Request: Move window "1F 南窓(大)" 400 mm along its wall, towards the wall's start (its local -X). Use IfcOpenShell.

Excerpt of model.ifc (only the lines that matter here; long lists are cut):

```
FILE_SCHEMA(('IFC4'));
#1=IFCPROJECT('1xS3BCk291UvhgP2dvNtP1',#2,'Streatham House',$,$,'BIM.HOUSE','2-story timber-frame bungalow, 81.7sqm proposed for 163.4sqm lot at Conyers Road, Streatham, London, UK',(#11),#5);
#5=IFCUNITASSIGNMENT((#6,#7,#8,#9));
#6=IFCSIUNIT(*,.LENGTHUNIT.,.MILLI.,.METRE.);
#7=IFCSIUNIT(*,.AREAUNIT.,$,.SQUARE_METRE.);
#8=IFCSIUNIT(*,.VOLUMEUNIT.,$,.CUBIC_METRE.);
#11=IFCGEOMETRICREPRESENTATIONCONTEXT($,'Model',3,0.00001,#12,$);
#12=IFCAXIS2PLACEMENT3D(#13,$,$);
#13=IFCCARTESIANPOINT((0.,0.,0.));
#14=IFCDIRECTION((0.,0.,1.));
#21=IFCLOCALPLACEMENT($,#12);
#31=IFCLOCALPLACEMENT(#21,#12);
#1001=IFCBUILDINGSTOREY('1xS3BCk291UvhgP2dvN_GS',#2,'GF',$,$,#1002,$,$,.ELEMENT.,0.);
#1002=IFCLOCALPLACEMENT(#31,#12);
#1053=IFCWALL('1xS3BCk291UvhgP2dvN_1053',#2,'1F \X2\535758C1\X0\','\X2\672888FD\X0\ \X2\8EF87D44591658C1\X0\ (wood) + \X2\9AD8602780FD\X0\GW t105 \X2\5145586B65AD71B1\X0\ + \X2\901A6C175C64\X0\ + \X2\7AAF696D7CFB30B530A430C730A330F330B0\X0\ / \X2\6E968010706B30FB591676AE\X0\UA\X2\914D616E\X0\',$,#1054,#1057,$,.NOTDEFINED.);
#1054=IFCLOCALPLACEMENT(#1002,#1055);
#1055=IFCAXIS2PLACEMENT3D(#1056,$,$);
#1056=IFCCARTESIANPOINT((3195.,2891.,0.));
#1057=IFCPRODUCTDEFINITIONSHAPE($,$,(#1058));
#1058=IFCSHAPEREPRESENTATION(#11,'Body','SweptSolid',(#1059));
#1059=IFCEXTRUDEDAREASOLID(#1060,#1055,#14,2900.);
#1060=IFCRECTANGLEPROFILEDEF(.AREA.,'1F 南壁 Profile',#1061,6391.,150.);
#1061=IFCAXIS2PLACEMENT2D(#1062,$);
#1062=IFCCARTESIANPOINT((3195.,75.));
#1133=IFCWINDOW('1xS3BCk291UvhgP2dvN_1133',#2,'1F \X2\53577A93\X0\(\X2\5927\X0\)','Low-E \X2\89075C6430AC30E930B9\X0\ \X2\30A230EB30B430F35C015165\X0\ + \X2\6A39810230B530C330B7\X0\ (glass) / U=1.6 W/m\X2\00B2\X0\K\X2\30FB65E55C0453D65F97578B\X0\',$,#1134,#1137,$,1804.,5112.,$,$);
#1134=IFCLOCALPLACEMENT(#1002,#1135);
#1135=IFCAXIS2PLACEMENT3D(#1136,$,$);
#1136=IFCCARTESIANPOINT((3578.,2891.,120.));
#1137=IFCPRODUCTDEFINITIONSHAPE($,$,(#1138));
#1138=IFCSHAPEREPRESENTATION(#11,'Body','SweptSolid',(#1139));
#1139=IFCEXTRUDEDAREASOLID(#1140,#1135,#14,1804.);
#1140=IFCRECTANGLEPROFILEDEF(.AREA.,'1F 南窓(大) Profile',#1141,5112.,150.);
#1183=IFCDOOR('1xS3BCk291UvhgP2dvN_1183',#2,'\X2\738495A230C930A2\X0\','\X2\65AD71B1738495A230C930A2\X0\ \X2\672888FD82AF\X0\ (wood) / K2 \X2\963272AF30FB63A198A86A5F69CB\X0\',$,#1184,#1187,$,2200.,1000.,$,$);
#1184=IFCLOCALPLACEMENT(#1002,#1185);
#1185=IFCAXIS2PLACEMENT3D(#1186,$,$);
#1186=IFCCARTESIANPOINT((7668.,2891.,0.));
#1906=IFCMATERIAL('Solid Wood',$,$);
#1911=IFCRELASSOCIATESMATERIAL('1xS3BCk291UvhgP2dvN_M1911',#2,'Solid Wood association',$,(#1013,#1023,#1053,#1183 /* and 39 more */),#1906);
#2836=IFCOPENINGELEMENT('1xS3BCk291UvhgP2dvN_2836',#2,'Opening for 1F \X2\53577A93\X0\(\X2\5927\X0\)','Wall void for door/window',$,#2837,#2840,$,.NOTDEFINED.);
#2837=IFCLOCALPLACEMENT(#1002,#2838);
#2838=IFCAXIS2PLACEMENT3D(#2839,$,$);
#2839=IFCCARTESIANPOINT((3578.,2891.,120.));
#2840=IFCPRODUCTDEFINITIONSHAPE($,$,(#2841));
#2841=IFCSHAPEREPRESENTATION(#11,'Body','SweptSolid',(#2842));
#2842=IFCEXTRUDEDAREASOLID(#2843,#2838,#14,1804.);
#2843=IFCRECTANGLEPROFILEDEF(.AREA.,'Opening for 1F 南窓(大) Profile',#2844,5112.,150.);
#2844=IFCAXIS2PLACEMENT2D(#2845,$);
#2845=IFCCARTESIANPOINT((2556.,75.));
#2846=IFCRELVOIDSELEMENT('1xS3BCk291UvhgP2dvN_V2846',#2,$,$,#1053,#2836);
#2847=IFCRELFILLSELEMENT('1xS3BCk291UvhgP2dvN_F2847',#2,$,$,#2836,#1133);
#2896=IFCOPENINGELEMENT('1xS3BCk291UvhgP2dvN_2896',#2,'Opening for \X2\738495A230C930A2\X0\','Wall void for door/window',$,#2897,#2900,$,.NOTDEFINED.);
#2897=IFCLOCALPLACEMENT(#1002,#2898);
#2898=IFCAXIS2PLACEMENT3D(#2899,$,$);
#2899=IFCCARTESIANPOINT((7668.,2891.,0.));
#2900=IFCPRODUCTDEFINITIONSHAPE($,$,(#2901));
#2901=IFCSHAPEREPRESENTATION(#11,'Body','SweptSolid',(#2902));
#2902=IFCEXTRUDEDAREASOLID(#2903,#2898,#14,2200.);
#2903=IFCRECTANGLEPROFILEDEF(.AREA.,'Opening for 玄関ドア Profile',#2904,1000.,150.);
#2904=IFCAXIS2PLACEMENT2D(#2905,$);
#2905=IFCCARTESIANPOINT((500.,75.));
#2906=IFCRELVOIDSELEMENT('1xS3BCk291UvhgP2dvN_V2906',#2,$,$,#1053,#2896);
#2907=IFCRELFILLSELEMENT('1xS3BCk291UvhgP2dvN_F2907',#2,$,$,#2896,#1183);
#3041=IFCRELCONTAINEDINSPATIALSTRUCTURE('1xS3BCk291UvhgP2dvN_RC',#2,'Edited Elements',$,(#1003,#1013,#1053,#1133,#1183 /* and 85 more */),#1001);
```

```python
import ifcopenshell
import ifcopenshell.api.geometry
import ifcopenshell.util.placement
import ifcopenshell.util.unit

model = ifcopenshell.open("model.ifc")
unit_scale = ifcopenshell.util.unit.calculate_unit_scale(model)

window = model.by_id(1133)
opening = window.FillsVoids[0].RelatingOpeningElement
wall = opening.VoidsElements[0].RelatingBuildingElement

wall_matrix = ifcopenshell.util.placement.get_local_placement(wall.ObjectPlacement)
shift = wall_matrix[:3, 0] * -0.4 / unit_scale
before = ifcopenshell.util.placement.get_local_placement(window.ObjectPlacement)[:3, 3].copy()

# The window is not placed relative to its opening, so move both.
for product in (opening, window):
    matrix = ifcopenshell.util.placement.get_local_placement(product.ObjectPlacement)
    matrix[:3, 3] += shift
    ifcopenshell.api.geometry.edit_object_placement(model, product=product, matrix=matrix, is_si=False)

after = ifcopenshell.util.placement.get_local_placement(window.ObjectPlacement)[:3, 3]
print("window moved by", (after - before).round(3) + 0.0)

model.write("model_edited.ifc")
```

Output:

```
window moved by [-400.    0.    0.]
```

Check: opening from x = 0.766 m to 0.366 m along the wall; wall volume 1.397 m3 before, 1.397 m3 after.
